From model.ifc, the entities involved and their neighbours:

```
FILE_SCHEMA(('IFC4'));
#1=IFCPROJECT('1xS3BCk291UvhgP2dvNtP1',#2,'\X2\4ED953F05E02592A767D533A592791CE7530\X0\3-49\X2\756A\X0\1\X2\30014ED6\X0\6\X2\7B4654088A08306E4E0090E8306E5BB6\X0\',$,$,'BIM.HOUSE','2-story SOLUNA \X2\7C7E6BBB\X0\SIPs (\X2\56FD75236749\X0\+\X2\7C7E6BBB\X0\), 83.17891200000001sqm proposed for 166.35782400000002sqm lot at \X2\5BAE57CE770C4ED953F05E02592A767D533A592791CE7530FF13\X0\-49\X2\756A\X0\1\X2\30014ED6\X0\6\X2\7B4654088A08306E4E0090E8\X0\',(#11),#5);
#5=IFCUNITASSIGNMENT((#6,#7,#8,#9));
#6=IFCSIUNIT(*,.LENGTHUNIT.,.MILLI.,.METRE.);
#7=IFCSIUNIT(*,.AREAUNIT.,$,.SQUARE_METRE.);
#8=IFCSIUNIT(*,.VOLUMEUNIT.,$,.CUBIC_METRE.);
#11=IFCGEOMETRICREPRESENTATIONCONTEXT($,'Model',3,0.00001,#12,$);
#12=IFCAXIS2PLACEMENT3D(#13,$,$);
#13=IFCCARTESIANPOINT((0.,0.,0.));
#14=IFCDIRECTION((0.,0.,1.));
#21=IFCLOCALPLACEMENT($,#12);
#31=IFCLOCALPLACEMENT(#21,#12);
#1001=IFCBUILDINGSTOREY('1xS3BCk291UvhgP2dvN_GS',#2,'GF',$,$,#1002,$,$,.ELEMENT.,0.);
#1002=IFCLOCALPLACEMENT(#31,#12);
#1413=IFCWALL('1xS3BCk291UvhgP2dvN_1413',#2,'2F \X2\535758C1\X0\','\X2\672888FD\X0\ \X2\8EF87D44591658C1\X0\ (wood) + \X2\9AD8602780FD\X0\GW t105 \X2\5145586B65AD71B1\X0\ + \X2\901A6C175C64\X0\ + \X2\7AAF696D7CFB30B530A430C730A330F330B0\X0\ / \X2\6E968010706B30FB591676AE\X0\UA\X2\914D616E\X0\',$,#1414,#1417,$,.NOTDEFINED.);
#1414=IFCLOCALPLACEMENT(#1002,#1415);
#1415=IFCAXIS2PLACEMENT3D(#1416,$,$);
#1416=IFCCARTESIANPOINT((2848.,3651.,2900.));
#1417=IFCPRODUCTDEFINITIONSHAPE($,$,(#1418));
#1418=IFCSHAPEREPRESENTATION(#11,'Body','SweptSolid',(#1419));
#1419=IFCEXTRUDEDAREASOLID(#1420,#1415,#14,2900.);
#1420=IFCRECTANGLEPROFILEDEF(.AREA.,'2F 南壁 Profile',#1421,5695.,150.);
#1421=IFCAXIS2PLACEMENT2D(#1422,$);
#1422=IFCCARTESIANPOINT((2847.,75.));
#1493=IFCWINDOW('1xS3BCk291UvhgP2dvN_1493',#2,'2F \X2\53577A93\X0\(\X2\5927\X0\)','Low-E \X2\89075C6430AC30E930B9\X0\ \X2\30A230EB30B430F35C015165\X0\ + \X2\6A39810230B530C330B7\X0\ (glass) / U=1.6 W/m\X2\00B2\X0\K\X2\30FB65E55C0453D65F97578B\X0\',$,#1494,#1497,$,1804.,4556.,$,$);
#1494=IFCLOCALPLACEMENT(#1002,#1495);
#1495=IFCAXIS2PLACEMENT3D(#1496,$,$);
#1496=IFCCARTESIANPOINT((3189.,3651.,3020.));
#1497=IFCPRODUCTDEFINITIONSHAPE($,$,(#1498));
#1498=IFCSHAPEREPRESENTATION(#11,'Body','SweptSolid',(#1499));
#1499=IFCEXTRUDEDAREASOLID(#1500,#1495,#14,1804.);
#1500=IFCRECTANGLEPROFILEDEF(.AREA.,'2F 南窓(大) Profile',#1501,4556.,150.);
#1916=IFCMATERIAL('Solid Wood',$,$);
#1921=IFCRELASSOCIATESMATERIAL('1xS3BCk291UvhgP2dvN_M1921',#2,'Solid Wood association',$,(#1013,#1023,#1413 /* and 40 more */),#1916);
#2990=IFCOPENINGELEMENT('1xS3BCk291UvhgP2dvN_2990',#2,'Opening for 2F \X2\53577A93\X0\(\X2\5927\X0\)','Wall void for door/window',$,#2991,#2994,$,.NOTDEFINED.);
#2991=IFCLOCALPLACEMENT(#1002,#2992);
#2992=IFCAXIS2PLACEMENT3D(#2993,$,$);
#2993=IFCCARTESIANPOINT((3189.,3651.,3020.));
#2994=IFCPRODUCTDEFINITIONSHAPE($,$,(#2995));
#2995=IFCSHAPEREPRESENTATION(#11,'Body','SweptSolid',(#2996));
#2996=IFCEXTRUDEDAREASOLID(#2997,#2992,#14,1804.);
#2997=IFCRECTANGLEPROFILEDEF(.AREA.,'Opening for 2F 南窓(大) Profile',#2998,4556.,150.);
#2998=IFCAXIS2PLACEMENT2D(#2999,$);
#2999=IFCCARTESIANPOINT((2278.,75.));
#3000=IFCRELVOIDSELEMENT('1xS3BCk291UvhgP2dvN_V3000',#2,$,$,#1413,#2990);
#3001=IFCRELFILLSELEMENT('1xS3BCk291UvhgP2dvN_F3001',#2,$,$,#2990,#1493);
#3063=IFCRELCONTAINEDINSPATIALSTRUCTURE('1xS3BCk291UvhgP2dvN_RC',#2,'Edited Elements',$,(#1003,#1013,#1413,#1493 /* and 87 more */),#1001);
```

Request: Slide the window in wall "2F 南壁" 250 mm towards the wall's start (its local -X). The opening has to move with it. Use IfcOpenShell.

```python
import ifcopenshell
import ifcopenshell.api.geometry
import ifcopenshell.util.placement
import ifcopenshell.util.unit

model = ifcopenshell.open("model.ifc")
unit_scale = ifcopenshell.util.unit.calculate_unit_scale(model)

window = model.by_guid("1xS3BCk291UvhgP2dvN_1493")
opening = window.FillsVoids[0].RelatingOpeningElement
wall = opening.VoidsElements[0].RelatingBuildingElement

wall_matrix = ifcopenshell.util.placement.get_local_placement(wall.ObjectPlacement)
shift = wall_matrix[:3, 0] * -0.25 / unit_scale
before = ifcopenshell.util.placement.get_local_placement(window.ObjectPlacement)[:3, 3].copy()

# The window is not placed relative to its opening, so move both.
for product in (opening, window):
    matrix = ifcopenshell.util.placement.get_local_placement(product.ObjectPlacement)
    matrix[:3, 3] += shift
    ifcopenshell.api.geometry.edit_object_placement(model, product=product, matrix=matrix, is_si=False)

after = ifcopenshell.util.placement.get_local_placement(window.ObjectPlacement)[:3, 3]
print("window moved by", (after - before).round(3) + 0.0)

model.write("model-out.ifc")
```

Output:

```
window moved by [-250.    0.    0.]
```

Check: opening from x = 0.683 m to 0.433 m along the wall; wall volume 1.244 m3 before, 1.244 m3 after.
